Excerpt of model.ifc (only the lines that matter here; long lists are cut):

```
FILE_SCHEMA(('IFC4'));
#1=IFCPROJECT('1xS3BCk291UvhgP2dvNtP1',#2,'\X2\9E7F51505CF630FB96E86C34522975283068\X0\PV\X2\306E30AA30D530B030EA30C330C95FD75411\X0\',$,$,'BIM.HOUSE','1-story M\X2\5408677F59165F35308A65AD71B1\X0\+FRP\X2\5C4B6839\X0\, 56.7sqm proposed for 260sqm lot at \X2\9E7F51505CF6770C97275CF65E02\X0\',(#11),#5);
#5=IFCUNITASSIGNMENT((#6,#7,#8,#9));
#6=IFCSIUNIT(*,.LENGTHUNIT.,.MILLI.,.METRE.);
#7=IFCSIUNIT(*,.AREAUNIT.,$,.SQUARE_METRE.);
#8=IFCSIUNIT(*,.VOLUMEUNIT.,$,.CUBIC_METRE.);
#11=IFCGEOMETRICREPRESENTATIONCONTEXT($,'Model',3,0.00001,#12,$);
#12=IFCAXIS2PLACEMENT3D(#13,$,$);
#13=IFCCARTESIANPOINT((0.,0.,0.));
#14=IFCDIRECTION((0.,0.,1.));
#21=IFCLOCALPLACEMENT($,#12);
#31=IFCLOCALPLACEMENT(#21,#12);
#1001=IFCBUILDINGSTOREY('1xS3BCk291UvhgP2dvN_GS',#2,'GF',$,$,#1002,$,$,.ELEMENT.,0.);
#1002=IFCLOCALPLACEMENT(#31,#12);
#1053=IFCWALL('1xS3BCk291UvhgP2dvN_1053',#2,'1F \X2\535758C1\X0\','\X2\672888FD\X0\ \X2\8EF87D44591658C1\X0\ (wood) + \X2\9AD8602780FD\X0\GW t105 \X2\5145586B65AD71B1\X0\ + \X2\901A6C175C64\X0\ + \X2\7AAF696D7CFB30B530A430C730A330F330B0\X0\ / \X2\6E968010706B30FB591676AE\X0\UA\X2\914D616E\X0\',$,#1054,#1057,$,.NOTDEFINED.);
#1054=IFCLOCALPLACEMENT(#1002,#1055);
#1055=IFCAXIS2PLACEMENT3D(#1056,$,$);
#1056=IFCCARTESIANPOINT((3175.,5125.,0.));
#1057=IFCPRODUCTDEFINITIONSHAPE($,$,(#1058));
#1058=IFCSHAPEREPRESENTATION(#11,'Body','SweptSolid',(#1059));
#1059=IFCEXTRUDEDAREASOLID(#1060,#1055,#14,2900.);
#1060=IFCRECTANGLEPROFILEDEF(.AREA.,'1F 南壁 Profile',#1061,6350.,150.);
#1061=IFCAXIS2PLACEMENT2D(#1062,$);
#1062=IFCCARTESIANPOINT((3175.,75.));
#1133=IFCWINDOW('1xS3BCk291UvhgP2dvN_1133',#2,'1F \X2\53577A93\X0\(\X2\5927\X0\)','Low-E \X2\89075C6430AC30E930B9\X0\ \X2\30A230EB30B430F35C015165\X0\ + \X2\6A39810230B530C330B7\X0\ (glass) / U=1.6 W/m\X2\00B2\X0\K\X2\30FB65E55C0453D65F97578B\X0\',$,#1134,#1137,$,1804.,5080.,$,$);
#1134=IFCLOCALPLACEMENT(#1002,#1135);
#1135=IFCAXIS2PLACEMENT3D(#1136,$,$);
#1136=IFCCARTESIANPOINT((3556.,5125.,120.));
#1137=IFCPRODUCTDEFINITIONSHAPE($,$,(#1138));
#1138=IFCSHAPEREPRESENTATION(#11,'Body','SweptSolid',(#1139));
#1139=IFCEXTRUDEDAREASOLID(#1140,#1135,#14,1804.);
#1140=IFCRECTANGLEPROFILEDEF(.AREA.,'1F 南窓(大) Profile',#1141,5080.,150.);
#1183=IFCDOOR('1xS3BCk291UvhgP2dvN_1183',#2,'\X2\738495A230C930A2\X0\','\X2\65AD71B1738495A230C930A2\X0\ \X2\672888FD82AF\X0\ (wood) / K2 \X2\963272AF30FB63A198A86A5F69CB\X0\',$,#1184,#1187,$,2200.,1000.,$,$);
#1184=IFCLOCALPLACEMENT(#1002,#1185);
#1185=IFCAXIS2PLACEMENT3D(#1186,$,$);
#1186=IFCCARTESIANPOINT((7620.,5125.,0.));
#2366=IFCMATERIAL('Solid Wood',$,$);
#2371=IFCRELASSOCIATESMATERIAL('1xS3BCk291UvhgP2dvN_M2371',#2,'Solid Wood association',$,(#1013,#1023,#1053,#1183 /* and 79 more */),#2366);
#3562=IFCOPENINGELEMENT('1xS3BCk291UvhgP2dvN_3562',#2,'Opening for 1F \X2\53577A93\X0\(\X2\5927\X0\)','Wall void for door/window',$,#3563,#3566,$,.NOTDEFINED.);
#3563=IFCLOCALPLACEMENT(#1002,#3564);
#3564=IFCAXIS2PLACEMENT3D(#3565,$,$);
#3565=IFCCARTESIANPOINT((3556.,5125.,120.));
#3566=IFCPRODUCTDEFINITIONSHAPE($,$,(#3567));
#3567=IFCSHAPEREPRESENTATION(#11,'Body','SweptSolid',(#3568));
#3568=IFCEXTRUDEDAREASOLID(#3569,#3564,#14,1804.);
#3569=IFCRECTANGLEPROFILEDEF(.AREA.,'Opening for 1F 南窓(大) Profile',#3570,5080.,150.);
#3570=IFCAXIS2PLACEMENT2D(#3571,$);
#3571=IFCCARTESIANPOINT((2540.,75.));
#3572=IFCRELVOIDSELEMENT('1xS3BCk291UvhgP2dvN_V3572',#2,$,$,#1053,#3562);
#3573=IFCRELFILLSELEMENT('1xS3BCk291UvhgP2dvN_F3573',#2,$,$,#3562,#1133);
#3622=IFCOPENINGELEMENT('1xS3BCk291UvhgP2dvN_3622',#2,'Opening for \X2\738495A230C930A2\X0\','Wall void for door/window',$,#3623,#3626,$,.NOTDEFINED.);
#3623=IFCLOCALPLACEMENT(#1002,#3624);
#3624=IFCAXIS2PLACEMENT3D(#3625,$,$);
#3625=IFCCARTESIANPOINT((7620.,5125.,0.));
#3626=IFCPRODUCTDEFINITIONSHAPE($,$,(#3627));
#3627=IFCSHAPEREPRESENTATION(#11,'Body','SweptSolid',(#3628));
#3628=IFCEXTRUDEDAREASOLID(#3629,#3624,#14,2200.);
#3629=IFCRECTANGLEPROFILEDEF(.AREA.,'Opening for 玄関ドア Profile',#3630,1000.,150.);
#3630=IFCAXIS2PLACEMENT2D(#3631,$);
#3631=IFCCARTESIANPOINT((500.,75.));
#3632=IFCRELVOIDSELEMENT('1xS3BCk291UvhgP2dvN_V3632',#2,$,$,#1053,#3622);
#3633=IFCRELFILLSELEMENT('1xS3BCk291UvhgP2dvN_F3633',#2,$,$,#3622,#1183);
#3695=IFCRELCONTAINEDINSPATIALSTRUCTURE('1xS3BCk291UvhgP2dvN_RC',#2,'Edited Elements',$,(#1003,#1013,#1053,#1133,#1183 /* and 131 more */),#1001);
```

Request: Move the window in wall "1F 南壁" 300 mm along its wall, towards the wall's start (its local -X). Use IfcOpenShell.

```python
import ifcopenshell
import ifcopenshell.api.geometry
import ifcopenshell.util.placement

model = ifcopenshell.open("model.ifc")

window = model.by_id(1133)
opening = window.FillsVoids[0].RelatingOpeningElement
wall = opening.VoidsElements[0].RelatingBuildingElement

wall_matrix = ifcopenshell.util.placement.get_local_placement(wall.ObjectPlacement)
shift = wall_matrix[:3, 0] * -300.0
before = ifcopenshell.util.placement.get_local_placement(window.ObjectPlacement)[:3, 3].copy()

# The window is not placed relative to its opening, so move both.
for product in (opening, window):
    matrix = ifcopenshell.util.placement.get_local_placement(product.ObjectPlacement)
    matrix[:3, 3] += shift
    ifcopenshell.api.geometry.edit_object_placement(model, product=product, matrix=matrix, is_si=False)

after = ifcopenshell.util.placement.get_local_placement(window.ObjectPlacement)[:3, 3]
print("window moved by", (after - before).round(3) + 0.0)

model.write("model_updated.ifc")
```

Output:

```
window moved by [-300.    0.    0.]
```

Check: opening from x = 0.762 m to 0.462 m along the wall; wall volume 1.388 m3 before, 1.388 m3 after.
